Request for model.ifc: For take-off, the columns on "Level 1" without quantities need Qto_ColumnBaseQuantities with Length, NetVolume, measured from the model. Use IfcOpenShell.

First a look at what the model holds.

```python
import ifcopenshell
import ifcopenshell.util.element
import ifcopenshell.util.unit

model = ifcopenshell.open("model.ifc")
print(model.schema)
for unit_type in ("LENGTHUNIT", "AREAUNIT", "VOLUMEUNIT"):
    print(unit_type, ifcopenshell.util.unit.calculate_unit_scale(model, unit_type))
storey = next(s for s in model.by_type("IfcBuildingStorey") if s.Name == "Level 1")
columns = [e for e in ifcopenshell.util.element.get_decomposition(storey) if e.is_a("IfcColumn")]
for e in sorted(columns, key=lambda e: e.id()):
    print(e.id(), e.is_a(), e.Name, list(ifcopenshell.util.element.get_psets(e, qtos_only=True)), sep=" | ")
```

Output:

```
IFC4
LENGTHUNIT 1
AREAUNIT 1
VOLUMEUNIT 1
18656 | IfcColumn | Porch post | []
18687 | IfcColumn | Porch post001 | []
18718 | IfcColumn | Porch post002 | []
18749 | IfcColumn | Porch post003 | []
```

```python
import ifcopenshell
import ifcopenshell.api.pset
import ifcopenshell.geom
import ifcopenshell.util.element
import ifcopenshell.util.shape
import ifcopenshell.util.unit

model = ifcopenshell.open("model.ifc")
unit_scale = ifcopenshell.util.unit.calculate_unit_scale(model)
volume_scale = ifcopenshell.util.unit.calculate_unit_scale(model, "VOLUMEUNIT")
settings = ifcopenshell.geom.settings()

storey = next(s for s in model.by_type("IfcBuildingStorey") if s.Name == "Level 1")
columns = [e for e in ifcopenshell.util.element.get_decomposition(storey) if e.is_a("IfcColumn")]

for e in sorted(columns, key=lambda e: e.id()):
    if ifcopenshell.util.element.get_psets(e, qtos_only=True, should_inherit=False):
        continue
    # Geometry comes back in metres, in the element's own axes.
    shape = ifcopenshell.geom.create_shape(settings, e)
    values = {
        "Length": ifcopenshell.util.shape.get_z(shape.geometry) / unit_scale,
        "NetVolume": ifcopenshell.util.shape.get_volume(shape.geometry) / volume_scale,
    }
    qto = ifcopenshell.api.pset.add_qto(model, product=e, name="Qto_ColumnBaseQuantities")
    ifcopenshell.api.pset.edit_qto(model, qto=qto, properties=values)
    print(e.id(), {k: round(v, 3) for k, v in values.items()})

model.write("model-out.ifc")
```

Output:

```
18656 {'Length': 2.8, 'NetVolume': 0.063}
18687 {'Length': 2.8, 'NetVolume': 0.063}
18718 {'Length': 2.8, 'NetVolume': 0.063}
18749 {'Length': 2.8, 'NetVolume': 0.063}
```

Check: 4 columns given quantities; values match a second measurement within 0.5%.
